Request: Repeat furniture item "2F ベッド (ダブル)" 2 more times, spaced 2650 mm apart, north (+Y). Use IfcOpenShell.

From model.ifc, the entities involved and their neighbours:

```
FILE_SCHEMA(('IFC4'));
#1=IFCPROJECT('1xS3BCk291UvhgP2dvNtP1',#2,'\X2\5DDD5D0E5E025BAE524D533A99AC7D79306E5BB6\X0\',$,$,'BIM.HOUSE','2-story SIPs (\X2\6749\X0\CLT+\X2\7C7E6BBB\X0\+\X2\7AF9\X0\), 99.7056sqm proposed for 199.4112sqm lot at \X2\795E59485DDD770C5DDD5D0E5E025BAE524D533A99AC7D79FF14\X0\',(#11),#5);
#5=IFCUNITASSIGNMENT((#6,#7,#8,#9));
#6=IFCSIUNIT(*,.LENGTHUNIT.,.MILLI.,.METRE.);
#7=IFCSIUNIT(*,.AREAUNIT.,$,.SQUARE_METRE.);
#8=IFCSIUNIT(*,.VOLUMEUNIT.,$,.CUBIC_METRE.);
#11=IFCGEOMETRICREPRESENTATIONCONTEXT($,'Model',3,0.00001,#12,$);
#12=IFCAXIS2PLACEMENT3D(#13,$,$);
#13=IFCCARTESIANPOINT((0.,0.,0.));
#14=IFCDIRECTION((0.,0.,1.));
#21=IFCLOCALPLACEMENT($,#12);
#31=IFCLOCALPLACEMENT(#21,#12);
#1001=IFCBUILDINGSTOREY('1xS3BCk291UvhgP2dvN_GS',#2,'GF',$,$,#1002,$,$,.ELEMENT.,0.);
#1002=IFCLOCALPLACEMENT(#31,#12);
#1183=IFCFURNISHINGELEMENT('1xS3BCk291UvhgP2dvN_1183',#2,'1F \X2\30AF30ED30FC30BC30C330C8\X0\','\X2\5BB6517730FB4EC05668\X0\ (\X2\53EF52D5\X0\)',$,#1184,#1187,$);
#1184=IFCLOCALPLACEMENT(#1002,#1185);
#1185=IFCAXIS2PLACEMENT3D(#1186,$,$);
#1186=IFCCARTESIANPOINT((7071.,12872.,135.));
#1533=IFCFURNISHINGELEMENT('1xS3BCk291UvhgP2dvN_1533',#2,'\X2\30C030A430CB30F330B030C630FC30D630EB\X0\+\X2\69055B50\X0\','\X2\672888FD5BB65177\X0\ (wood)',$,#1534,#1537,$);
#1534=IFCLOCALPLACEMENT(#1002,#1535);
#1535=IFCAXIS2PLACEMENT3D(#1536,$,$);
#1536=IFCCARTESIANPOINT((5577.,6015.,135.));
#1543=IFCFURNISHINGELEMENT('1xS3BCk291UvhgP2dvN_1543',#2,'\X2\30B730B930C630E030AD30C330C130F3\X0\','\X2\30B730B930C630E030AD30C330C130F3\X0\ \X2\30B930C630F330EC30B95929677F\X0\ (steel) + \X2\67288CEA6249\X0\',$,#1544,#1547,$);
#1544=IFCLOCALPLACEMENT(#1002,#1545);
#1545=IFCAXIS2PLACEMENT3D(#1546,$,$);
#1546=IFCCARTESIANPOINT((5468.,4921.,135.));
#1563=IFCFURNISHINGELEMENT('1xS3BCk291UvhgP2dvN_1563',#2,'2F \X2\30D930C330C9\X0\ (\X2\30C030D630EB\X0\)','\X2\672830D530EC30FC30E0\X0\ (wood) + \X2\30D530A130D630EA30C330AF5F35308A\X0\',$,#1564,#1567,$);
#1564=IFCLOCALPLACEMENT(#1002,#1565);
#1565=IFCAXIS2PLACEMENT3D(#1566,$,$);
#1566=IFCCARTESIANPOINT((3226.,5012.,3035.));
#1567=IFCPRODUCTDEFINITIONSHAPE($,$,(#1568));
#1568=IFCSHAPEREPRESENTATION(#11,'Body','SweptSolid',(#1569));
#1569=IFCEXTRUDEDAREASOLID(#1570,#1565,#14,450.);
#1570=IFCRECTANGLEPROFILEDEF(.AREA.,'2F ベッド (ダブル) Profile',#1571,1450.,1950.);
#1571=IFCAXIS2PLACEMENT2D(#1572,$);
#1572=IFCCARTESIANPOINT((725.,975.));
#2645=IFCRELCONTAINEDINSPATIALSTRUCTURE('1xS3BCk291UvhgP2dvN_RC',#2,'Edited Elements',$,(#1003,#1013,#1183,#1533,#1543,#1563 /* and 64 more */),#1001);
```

```python
import numpy as np
import ifcopenshell
import ifcopenshell.api.geometry
import ifcopenshell.api.root
import ifcopenshell.util.element
import ifcopenshell.util.placement

model = ifcopenshell.open("model.ifc")


def reuse_history(source, copy):
    """copy_class also copies each property set's owner history, people and application; keep the originals."""
    for rel in copy.IsDefinedBy:
        if rel.is_a("IfcRelDefinesByProperties") and (history := rel.RelatingPropertyDefinition.OwnerHistory):
            rel.RelatingPropertyDefinition.OwnerHistory = source.OwnerHistory
            ifcopenshell.util.element.remove_deep2(model, history)


source = model.by_guid("1xS3BCk291UvhgP2dvN_1563")
base = ifcopenshell.util.placement.get_local_placement(source.ObjectPlacement)
step = np.array([0.0, 1.0, 0.0]) * 2650.0

for i in range(1, 3):
    copy = ifcopenshell.api.root.copy_class(model, product=source)
    copy.Representation = ifcopenshell.util.element.copy_deep(
        model, source.Representation, exclude=["IfcGeometricRepresentationContext", "IfcRepresentationMap"]
    )
    reuse_history(source, copy)
    matrix = base.copy()
    matrix[:3, 3] += i * step
    print("added at", matrix[:3, 3].round(3) + 0.0)
    ifcopenshell.api.geometry.edit_object_placement(model, product=copy, matrix=matrix, is_si=False)

model.write("model_edited.ifc")
```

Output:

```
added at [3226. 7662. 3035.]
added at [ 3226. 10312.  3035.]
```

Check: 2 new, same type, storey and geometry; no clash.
